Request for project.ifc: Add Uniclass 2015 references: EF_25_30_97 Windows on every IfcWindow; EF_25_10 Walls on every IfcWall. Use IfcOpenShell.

First a look at what the model holds.

```python
import ifcopenshell

model = ifcopenshell.open("project.ifc")
print(model.schema)
print("classifications:", [c.Name for c in model.by_type("IfcClassification")])
for ifc_class in ("IfcDoor", "IfcRoof", "IfcStair", "IfcWall", "IfcWindow"):
    print(ifc_class, len(model.by_type(ifc_class)))
```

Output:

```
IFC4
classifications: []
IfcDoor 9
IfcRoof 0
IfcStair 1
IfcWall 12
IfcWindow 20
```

```python
import ifcopenshell
import ifcopenshell.api.classification

model = ifcopenshell.open("project.ifc")

system = ifcopenshell.api.classification.add_classification(model, classification="Uniclass 2015")

codes = {
    "IfcWindow": ("EF_25_30_97", "Windows"),
    "IfcWall": ("EF_25_10", "Walls"),
}
for ifc_class, (code, name) in codes.items():
    products = model.by_type(ifc_class)
    ifcopenshell.api.classification.add_reference(
        model, products=products, classification=system, identification=code, name=name
    )
    print(code, len(products))

model.write("project_updated.ifc")
```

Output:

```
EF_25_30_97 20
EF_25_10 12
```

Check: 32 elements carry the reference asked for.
